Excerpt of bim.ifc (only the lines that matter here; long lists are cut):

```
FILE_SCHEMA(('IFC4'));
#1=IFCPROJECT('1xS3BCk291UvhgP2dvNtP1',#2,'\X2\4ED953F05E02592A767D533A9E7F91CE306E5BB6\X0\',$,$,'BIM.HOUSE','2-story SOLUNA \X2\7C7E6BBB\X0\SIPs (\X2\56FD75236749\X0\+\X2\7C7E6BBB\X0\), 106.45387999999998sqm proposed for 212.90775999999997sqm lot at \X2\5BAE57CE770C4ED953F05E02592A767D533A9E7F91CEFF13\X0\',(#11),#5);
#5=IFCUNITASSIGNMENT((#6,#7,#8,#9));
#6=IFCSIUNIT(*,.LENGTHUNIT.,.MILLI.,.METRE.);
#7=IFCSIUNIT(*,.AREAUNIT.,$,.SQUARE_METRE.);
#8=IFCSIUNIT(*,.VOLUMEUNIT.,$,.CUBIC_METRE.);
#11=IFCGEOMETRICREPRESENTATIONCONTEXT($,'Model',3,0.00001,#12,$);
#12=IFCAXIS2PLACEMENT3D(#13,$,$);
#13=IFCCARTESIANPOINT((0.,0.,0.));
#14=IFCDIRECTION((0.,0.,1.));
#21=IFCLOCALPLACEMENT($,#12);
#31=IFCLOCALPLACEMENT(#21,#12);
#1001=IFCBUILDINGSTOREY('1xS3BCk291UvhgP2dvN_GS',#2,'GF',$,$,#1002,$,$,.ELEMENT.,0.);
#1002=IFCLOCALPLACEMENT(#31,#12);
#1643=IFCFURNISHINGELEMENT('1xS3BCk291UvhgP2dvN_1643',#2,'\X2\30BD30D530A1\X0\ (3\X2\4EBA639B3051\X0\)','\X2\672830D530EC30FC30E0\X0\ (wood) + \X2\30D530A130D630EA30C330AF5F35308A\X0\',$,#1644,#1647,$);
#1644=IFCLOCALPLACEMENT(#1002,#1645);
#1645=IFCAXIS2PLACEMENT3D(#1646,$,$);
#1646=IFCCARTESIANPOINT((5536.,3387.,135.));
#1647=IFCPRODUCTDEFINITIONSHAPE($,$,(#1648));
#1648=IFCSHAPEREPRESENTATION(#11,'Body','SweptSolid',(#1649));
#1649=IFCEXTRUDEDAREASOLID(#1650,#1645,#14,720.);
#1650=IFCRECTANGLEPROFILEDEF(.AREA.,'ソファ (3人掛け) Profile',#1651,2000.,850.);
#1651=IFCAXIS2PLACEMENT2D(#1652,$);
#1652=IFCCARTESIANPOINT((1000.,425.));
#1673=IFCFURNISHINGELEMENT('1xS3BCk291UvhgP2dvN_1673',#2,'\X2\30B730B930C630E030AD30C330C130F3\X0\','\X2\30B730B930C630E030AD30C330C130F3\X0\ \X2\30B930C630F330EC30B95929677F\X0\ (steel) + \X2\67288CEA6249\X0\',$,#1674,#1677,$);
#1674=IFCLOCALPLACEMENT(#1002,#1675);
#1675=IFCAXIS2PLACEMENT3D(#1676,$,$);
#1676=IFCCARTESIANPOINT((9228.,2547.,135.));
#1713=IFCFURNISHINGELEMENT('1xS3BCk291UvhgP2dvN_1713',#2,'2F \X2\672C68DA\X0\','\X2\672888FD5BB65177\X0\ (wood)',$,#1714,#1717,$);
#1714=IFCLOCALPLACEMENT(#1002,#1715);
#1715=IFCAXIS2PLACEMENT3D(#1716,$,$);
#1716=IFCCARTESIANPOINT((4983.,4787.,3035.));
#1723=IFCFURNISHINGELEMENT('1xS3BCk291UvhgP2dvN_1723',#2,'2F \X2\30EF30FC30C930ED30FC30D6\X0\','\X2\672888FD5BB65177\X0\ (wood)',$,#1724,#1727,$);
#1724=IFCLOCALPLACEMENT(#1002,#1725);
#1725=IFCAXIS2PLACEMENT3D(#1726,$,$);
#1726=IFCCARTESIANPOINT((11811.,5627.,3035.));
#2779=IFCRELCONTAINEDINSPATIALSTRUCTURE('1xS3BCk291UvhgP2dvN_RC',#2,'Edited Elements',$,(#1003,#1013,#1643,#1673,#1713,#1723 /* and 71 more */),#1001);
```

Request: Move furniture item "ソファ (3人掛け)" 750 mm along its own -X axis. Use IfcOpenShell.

```python
import ifcopenshell
import ifcopenshell.api.geometry
import ifcopenshell.util.placement

model = ifcopenshell.open("bim.ifc")

item = model.by_id(1643)
matrix = ifcopenshell.util.placement.get_local_placement(item.ObjectPlacement)
matrix[:3, 3] -= matrix[:3, 0] * 750.0
ifcopenshell.api.geometry.edit_object_placement(model, product=item, matrix=matrix, is_si=False)

print(ifcopenshell.util.placement.get_local_placement(item.ObjectPlacement).round(3) + 0.0)

model.write("bim_edited.ifc")
```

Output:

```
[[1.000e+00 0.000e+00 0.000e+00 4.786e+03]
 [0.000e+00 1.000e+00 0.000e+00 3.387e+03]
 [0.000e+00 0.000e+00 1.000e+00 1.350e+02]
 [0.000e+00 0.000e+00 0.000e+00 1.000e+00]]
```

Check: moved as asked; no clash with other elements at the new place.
